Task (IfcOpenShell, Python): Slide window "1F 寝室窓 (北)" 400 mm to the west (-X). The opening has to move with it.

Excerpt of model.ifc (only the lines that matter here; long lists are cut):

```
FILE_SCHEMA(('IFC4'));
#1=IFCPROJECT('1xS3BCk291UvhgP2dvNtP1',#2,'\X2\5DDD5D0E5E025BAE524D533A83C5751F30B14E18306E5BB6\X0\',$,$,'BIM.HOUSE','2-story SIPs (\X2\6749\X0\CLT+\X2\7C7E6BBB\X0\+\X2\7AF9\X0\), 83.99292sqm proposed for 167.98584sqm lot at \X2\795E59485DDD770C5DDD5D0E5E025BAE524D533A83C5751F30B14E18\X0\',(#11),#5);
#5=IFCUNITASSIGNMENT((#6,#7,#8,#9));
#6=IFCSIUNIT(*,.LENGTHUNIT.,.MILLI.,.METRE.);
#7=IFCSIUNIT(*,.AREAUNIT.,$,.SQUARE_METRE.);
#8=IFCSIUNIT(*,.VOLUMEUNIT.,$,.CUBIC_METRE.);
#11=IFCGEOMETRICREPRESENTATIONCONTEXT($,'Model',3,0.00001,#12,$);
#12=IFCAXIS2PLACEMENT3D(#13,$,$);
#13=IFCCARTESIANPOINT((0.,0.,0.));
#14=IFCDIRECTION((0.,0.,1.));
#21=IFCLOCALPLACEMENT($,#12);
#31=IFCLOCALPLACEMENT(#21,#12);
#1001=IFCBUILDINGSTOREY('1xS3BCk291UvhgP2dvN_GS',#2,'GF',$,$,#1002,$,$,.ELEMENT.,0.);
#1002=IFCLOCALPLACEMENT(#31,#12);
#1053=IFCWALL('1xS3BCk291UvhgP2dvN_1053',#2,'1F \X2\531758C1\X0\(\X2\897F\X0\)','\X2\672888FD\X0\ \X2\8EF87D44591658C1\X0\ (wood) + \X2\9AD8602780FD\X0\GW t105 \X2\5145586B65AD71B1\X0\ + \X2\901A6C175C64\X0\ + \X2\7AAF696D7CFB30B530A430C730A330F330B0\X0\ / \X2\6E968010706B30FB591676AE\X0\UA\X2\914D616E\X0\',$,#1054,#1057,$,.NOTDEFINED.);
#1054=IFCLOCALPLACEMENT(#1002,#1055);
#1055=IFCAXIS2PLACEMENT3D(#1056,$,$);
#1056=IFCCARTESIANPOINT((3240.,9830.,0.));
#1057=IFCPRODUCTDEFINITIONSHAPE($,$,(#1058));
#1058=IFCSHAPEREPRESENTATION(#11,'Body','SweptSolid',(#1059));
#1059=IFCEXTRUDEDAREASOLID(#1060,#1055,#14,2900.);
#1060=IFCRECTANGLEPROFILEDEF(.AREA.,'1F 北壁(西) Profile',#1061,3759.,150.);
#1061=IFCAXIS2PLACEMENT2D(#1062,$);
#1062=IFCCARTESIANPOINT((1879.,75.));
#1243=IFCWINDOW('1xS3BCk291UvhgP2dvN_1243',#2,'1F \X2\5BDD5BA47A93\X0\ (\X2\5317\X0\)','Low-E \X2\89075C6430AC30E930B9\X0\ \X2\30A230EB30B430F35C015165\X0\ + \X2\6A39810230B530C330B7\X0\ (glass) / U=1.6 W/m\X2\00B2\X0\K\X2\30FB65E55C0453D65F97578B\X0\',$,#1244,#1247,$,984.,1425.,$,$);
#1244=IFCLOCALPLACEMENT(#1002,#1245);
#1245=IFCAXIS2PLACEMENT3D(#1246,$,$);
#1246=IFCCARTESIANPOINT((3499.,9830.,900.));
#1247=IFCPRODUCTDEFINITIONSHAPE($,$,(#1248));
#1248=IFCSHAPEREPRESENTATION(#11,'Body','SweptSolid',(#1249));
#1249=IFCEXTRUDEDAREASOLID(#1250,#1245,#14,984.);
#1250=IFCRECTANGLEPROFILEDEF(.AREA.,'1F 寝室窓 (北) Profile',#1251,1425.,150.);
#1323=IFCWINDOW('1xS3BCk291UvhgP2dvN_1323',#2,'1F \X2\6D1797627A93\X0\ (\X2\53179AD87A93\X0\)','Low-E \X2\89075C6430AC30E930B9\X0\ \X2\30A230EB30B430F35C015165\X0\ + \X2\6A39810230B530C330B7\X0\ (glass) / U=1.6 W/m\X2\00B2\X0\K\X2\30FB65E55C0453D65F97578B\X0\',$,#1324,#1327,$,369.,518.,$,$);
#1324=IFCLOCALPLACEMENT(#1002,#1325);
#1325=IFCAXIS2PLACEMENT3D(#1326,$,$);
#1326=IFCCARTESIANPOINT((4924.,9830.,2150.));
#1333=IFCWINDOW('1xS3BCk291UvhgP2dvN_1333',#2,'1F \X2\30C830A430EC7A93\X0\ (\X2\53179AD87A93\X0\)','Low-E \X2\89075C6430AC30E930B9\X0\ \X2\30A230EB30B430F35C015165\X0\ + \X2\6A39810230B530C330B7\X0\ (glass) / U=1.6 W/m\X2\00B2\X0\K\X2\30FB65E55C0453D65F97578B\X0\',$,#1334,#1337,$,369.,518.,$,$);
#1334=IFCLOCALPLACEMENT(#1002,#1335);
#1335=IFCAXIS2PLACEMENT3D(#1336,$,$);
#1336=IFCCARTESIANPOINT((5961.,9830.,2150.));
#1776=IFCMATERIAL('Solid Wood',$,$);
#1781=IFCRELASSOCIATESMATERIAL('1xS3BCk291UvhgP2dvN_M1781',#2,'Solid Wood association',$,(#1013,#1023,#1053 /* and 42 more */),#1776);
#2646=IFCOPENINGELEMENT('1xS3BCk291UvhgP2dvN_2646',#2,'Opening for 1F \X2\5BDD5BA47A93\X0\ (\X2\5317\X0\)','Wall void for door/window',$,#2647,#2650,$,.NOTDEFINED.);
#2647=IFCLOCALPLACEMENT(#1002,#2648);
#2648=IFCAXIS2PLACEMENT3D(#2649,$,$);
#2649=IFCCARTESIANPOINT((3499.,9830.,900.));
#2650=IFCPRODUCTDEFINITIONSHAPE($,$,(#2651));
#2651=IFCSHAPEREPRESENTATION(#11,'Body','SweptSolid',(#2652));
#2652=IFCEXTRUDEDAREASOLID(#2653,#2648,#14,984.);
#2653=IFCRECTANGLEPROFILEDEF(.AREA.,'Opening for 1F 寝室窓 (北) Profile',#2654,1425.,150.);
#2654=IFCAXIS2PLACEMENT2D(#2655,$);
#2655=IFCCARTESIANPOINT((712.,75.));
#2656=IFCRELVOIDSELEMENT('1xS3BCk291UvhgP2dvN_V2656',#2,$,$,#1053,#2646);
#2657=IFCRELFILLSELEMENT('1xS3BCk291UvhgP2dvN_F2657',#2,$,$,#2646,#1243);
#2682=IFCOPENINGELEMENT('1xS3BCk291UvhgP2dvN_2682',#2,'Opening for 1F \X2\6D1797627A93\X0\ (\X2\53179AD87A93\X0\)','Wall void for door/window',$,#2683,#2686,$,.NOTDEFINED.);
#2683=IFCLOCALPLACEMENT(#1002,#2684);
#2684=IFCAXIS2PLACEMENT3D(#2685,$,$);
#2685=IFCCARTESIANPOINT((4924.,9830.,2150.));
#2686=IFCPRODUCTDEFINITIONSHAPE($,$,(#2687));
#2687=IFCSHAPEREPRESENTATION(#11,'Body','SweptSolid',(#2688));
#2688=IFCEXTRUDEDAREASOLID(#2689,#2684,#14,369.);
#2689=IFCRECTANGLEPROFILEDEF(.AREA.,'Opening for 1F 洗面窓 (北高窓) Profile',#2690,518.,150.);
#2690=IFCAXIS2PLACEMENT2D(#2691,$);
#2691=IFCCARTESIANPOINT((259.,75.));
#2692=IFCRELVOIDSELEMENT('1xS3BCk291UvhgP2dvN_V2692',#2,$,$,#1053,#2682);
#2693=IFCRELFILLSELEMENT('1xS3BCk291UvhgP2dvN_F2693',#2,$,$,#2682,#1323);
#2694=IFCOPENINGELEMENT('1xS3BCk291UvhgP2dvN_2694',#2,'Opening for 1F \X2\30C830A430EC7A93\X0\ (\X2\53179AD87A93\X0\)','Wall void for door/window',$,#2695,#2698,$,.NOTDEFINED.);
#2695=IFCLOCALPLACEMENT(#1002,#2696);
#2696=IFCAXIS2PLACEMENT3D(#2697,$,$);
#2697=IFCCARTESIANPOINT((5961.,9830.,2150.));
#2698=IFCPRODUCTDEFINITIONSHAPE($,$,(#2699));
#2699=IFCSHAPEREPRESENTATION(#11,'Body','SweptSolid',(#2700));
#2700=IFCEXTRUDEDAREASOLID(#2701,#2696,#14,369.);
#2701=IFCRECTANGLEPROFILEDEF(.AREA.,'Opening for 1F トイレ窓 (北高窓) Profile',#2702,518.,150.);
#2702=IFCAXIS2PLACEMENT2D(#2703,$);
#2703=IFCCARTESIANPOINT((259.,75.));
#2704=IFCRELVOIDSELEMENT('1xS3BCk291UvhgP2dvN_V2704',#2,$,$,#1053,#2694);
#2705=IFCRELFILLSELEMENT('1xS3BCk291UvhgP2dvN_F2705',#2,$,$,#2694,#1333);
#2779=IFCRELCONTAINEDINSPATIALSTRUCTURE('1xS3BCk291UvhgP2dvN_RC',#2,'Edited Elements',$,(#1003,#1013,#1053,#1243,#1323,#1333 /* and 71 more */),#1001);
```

```python
import ifcopenshell
import ifcopenshell.api.geometry
import ifcopenshell.util.placement

model = ifcopenshell.open("model.ifc")

window = model.by_guid("1xS3BCk291UvhgP2dvN_1243")
opening = window.FillsVoids[0].RelatingOpeningElement
wall = opening.VoidsElements[0].RelatingBuildingElement

wall_matrix = ifcopenshell.util.placement.get_local_placement(wall.ObjectPlacement)
shift = wall_matrix[:3, 0] * -400.0
before = ifcopenshell.util.placement.get_local_placement(window.ObjectPlacement)[:3, 3].copy()

# The window is not placed relative to its opening, so move both.
for product in (opening, window):
    matrix = ifcopenshell.util.placement.get_local_placement(product.ObjectPlacement)
    matrix[:3, 3] += shift
    ifcopenshell.api.geometry.edit_object_placement(model, product=product, matrix=matrix, is_si=False)

after = ifcopenshell.util.placement.get_local_placement(window.ObjectPlacement)[:3, 3]
print("window moved by", (after - before).round(3) + 0.0)

model.write("model_rev.ifc")
```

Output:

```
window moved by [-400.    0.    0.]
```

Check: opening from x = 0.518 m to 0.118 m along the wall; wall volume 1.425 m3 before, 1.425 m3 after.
